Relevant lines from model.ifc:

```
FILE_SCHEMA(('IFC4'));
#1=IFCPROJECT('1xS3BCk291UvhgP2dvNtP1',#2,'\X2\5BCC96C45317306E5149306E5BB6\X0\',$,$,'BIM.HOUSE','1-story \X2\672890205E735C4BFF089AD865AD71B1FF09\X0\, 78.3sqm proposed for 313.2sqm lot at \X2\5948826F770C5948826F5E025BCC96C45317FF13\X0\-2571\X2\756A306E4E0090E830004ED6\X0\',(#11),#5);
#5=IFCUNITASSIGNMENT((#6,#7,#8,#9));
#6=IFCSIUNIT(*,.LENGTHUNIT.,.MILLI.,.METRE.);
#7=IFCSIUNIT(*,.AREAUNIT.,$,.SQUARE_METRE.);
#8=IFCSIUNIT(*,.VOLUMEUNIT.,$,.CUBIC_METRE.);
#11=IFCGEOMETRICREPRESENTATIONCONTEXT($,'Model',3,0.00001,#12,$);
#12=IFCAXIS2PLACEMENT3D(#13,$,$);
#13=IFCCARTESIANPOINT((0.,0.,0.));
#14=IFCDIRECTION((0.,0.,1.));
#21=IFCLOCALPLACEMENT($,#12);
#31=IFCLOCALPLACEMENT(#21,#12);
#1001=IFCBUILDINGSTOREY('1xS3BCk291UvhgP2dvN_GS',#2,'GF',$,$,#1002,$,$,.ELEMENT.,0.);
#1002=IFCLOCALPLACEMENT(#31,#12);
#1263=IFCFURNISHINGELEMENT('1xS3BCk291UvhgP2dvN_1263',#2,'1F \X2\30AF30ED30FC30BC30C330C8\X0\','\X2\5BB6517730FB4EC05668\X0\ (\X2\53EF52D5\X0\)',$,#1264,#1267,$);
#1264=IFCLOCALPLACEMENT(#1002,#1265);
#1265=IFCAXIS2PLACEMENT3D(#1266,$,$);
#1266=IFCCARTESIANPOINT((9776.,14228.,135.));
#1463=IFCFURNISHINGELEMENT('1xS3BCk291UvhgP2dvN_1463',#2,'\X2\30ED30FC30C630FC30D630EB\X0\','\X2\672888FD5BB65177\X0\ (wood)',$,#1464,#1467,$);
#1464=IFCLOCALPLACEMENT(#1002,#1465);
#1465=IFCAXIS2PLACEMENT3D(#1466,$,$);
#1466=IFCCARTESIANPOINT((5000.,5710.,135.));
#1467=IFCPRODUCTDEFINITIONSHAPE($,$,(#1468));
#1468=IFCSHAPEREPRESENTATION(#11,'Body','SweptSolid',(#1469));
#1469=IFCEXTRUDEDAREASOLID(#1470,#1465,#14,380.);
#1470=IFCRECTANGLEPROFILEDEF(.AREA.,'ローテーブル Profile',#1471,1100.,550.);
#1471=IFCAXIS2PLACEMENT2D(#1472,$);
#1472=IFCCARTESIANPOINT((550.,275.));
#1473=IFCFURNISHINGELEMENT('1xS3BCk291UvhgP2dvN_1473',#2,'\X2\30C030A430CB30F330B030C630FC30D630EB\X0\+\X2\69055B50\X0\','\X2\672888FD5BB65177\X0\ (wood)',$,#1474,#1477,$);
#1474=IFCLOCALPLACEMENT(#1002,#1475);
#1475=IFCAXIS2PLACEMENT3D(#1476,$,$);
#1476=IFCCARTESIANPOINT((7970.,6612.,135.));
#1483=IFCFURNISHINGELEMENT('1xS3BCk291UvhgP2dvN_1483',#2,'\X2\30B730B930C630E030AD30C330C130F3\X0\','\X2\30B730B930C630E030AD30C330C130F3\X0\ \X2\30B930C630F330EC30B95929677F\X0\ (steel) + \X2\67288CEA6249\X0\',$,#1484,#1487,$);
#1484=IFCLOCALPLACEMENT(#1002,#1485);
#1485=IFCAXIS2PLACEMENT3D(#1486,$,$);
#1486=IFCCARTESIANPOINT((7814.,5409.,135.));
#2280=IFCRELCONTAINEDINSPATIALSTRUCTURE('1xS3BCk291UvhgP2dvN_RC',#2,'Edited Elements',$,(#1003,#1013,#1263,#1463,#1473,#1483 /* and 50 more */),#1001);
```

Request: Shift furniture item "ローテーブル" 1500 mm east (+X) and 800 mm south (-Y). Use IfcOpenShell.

```python
import ifcopenshell
import ifcopenshell.api.geometry
import ifcopenshell.util.placement

model = ifcopenshell.open("model.ifc")

item = model.by_guid("1xS3BCk291UvhgP2dvN_1463")
matrix = ifcopenshell.util.placement.get_local_placement(item.ObjectPlacement)
matrix[0, 3] += 1500.0
matrix[1, 3] -= 800.0
ifcopenshell.api.geometry.edit_object_placement(model, product=item, matrix=matrix, is_si=False)

print(ifcopenshell.util.placement.get_local_placement(item.ObjectPlacement).round(3) + 0.0)

model.write("model_edited.ifc")
```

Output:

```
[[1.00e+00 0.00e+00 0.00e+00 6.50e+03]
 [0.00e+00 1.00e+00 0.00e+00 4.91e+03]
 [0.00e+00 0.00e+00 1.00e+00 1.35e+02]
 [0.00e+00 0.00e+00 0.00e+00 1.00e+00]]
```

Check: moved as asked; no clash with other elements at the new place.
